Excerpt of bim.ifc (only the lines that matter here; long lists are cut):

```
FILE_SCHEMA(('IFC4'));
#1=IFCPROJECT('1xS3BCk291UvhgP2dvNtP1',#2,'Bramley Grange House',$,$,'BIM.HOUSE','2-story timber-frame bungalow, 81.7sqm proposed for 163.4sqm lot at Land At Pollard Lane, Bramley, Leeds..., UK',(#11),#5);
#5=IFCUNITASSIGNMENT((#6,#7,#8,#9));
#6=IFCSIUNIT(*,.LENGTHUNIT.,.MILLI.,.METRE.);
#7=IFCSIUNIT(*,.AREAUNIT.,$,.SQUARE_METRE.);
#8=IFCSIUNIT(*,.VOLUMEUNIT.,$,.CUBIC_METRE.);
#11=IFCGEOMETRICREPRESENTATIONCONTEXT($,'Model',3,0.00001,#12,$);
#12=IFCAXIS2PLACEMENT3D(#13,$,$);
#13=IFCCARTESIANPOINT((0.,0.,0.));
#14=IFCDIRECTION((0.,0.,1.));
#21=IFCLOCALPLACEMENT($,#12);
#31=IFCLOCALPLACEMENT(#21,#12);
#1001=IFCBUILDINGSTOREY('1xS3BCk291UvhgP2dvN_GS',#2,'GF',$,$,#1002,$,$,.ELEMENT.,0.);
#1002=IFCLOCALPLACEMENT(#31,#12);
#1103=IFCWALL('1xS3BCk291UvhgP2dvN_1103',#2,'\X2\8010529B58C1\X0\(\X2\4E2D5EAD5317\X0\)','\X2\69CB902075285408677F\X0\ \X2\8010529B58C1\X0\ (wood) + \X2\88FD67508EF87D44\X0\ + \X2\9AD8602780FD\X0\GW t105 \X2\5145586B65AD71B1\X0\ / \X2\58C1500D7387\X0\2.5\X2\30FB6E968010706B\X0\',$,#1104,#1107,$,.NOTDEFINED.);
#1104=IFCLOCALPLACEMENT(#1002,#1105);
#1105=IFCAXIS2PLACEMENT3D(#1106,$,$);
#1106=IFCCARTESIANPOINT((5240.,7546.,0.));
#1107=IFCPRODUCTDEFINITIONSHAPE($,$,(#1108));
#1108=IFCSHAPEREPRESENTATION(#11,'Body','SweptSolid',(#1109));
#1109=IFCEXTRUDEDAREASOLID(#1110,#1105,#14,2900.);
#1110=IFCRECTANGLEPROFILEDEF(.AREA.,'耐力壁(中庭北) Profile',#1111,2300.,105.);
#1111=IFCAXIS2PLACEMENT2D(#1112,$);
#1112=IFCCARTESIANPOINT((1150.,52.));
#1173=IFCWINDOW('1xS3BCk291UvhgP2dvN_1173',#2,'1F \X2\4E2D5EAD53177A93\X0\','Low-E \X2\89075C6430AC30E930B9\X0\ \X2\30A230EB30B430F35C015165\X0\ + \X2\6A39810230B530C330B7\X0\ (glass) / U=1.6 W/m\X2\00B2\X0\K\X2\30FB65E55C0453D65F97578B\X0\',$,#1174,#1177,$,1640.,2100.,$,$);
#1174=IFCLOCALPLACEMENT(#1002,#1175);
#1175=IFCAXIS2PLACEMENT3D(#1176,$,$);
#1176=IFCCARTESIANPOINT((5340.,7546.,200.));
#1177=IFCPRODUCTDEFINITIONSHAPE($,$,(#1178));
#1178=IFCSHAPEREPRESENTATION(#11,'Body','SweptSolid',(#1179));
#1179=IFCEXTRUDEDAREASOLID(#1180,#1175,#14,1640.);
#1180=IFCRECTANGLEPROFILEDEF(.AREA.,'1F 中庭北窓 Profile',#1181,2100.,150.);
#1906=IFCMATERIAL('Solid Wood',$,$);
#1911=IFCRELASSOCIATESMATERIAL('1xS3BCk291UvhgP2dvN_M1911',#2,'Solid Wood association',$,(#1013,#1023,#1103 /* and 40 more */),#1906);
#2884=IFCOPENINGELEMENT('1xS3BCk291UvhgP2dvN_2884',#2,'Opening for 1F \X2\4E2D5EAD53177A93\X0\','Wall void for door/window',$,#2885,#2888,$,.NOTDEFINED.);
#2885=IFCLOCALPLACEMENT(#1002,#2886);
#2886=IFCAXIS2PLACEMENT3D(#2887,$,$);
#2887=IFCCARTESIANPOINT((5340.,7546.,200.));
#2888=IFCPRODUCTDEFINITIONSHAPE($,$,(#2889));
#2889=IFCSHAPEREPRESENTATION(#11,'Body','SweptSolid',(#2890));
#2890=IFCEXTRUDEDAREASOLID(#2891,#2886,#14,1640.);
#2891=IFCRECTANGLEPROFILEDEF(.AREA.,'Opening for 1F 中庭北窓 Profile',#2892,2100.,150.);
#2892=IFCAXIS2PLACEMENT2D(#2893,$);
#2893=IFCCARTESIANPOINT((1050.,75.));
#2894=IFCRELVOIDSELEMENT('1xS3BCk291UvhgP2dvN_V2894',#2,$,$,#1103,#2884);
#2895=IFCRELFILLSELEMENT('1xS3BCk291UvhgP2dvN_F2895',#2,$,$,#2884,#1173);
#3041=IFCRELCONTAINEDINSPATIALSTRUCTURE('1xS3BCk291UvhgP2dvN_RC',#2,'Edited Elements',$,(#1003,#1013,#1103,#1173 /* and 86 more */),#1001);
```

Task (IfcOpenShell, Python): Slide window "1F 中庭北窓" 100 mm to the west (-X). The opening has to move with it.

```python
import ifcopenshell
import ifcopenshell.api.geometry
import ifcopenshell.util.placement

model = ifcopenshell.open("bim.ifc")

window = model.by_guid("1xS3BCk291UvhgP2dvN_1173")
opening = window.FillsVoids[0].RelatingOpeningElement
wall = opening.VoidsElements[0].RelatingBuildingElement

wall_matrix = ifcopenshell.util.placement.get_local_placement(wall.ObjectPlacement)
shift = wall_matrix[:3, 0] * -100.0
before = ifcopenshell.util.placement.get_local_placement(window.ObjectPlacement)[:3, 3].copy()

# The window is not placed relative to its opening, so move both.
for product in (opening, window):
    matrix = ifcopenshell.util.placement.get_local_placement(product.ObjectPlacement)
    matrix[:3, 3] += shift
    ifcopenshell.api.geometry.edit_object_placement(model, product=product, matrix=matrix, is_si=False)

after = ifcopenshell.util.placement.get_local_placement(window.ObjectPlacement)[:3, 3]
print("window moved by", (after - before).round(3) + 0.0)

model.write("bim_updated.ifc")
```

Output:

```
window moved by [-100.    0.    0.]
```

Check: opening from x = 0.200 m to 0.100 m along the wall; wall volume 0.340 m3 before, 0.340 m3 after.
